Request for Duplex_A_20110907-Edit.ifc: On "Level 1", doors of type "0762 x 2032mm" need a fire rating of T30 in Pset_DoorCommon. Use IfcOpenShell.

First a look at what the model holds.

```python
import ifcopenshell
import ifcopenshell.util.element

model = ifcopenshell.open("Duplex_A_20110907-Edit.ifc")
print(model.schema)
storey = next(s for s in model.by_type("IfcBuildingStorey") if s.Name == "Level 1")
doors = [e for e in ifcopenshell.util.element.get_decomposition(storey) if e.is_a("IfcDoor")]
seen = {}
for e in doors:
    element_type = ifcopenshell.util.element.get_type(e)
    key = (element_type.Name if element_type != e and element_type else None, ifcopenshell.util.element.get_pset(e, "Pset_DoorCommon", "FireRating"))
    seen[key] = seen.get(key, 0) + 1
for (name, value), count in sorted(seen.items(), key=str):
    print(count, "x", name, "|", value)
```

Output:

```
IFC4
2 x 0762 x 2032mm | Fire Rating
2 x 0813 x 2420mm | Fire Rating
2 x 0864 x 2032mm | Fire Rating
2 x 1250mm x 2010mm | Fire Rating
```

```python
import ifcopenshell
import ifcopenshell.api.pset
import ifcopenshell.util.element

model = ifcopenshell.open("Duplex_A_20110907-Edit.ifc")

storey = next(s for s in model.by_type("IfcBuildingStorey") if s.Name == "Level 1")
doors = [e for e in ifcopenshell.util.element.get_decomposition(storey) if e.is_a("IfcDoor")]

count = 0
for e in doors:
    element_type = ifcopenshell.util.element.get_type(e)
    if element_type in (None, e) or element_type.Name != "0762 x 2032mm":
        continue
    # add_pset returns the element's existing set when there is one.
    pset = ifcopenshell.api.pset.add_pset(model, product=e, name="Pset_DoorCommon")
    ifcopenshell.api.pset.edit_pset(model, pset=pset, properties={"FireRating": "T30"})
    count += 1

print(count, "doors updated")

model.write("Duplex_A_20110907-Edit-out.ifc")
```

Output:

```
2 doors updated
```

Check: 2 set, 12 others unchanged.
